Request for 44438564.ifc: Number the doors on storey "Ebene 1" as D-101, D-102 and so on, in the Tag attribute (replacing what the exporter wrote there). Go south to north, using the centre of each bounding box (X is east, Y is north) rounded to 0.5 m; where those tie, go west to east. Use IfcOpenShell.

First a look at what the model holds.

```python
import ifcopenshell
import ifcopenshell.util.element
import ifcopenshell.util.placement

model = ifcopenshell.open("44438564.ifc")
print(model.schema)
storey = next(s for s in model.by_type("IfcBuildingStorey") if s.Name == "Ebene 1")
doors = [e for e in ifcopenshell.util.element.get_decomposition(storey) if e.is_a("IfcDoor")]
for e in sorted(doors, key=lambda e: e.id()):
    origin = ifcopenshell.util.placement.get_local_placement(e.ObjectPlacement)[:3, 3]
    print(e.id(), e.Tag, e.Name, origin.round(2) + 0.0, sep=" | ")
```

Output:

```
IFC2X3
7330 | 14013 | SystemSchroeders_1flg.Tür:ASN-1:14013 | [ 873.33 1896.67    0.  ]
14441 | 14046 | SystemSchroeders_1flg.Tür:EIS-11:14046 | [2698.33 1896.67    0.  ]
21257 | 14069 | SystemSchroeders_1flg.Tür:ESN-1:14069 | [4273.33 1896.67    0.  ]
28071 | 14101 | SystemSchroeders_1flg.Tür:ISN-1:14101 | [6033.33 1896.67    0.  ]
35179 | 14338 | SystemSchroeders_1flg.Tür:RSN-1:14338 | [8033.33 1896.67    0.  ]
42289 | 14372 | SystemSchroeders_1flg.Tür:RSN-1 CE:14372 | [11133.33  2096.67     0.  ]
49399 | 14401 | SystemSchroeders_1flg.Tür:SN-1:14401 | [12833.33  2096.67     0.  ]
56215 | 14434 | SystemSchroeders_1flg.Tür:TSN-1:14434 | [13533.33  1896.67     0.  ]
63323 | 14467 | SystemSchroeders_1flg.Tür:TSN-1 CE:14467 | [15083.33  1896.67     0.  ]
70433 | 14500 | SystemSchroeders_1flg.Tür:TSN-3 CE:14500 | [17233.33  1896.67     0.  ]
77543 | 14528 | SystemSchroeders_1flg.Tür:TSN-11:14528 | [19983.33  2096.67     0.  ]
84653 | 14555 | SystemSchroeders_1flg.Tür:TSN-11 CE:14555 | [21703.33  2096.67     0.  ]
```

```python
import ifcopenshell
import ifcopenshell.geom
import ifcopenshell.util.element
import ifcopenshell.util.shape

model = ifcopenshell.open("44438564.ifc")
settings = ifcopenshell.geom.settings()
settings.set("use-world-coords", True)


def centre(element):
    shape = ifcopenshell.geom.create_shape(settings, element)
    return ifcopenshell.util.shape.get_bbox_centroid(shape.geometry)


storey = next(s for s in model.by_type("IfcBuildingStorey") if s.Name == "Ebene 1")
doors = [e for e in ifcopenshell.util.element.get_decomposition(storey) if e.is_a("IfcDoor")]

# Insertion points can sit at a corner or the storey origin, so sort by the geometry (in metres).
centres = {e: centre(e) for e in doors}
doors.sort(key=lambda e: (round(centres[e][1] / 0.5), centres[e][0]))

for i, e in enumerate(doors, start=1):
    number = f"D-1{i:02d}"
    e.Tag = number
    print(e.id(), number)

model.write("44438564-out.ifc")
```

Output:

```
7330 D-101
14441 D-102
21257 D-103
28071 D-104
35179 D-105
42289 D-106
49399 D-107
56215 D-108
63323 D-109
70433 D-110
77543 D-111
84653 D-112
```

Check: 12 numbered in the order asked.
